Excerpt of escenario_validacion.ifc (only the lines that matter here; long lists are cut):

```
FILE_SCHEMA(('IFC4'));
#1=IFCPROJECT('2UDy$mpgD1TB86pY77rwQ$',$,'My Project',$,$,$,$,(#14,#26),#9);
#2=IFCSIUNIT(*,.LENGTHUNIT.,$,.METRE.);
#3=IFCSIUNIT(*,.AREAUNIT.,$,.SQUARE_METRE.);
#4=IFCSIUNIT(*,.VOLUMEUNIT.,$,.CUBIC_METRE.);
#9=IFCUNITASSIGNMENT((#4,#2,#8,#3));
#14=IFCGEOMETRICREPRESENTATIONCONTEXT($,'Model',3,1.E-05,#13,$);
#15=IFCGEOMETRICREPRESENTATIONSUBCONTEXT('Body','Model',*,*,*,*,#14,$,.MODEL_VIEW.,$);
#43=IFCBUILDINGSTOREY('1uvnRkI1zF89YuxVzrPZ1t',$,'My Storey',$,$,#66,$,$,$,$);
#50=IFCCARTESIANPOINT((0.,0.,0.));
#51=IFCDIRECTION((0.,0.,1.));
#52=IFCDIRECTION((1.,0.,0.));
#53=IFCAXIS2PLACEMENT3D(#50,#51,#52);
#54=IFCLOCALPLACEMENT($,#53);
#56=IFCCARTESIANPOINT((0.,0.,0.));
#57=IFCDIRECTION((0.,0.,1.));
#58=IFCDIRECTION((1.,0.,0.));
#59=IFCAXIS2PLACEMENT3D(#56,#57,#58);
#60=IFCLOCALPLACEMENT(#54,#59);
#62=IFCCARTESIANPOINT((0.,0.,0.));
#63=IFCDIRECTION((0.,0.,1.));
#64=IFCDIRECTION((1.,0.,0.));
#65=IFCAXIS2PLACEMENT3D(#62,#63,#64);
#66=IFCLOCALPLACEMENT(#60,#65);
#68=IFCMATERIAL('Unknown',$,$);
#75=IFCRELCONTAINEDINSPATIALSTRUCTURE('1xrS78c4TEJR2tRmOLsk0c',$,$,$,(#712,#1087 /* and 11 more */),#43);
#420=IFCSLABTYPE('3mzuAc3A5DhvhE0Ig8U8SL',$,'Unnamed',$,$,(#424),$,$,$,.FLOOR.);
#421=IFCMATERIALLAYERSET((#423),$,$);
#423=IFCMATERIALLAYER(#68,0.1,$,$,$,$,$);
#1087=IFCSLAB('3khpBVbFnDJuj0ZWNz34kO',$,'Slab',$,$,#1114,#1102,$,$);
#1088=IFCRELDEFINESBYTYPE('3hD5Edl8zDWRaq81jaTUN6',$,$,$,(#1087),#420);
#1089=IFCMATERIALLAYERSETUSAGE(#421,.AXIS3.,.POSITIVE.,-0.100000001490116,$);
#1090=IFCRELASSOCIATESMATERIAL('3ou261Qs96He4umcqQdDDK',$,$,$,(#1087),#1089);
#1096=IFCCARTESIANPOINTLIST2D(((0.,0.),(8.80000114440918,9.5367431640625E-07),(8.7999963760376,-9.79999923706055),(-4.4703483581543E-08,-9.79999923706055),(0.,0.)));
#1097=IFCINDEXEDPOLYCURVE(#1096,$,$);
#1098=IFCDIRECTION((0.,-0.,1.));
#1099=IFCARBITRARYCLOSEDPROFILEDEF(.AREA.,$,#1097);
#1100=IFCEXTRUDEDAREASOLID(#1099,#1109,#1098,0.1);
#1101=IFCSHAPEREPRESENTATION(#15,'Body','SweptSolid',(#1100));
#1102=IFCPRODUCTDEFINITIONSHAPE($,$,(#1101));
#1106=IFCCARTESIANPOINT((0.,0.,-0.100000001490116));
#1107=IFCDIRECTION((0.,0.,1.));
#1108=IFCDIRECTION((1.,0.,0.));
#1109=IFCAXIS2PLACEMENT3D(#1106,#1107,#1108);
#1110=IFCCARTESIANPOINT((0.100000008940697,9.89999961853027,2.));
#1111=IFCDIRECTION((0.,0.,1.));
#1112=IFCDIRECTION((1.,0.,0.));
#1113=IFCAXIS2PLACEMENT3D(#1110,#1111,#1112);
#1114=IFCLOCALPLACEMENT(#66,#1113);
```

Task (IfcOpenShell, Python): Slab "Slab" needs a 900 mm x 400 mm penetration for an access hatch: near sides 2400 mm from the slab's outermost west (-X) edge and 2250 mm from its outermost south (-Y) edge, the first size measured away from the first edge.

```python
import numpy as np
import ifcopenshell
import ifcopenshell.api.feature
import ifcopenshell.api.geometry
import ifcopenshell.api.root
import ifcopenshell.geom
import ifcopenshell.util.placement
import ifcopenshell.util.representation
import ifcopenshell.util.shape
import ifcopenshell.util.unit

model = ifcopenshell.open("escenario_validacion.ifc")
unit_scale = ifcopenshell.util.unit.calculate_unit_scale(model)
settings = ifcopenshell.geom.settings()


def volume(element):
    """Net volume in cubic metres, openings subtracted."""
    shape = ifcopenshell.geom.create_shape(settings, element)
    return ifcopenshell.util.shape.get_volume(shape.geometry)


slab = model.by_id(1087)
before = volume(slab)

# Extent in the slab's own axes, in metres. The edges named are its -X and -Y sides.
slab_shape = ifcopenshell.geom.create_shape(settings, slab)
vertices = ifcopenshell.util.shape.get_vertices(slab_shape.geometry)
x_min, y_min, bottom = vertices.min(axis=0)
top = vertices[:, 2].max()

opening = ifcopenshell.api.root.create_entity(model, ifc_class="IfcOpeningElement", name="Access hatch opening", predefined_type="OPENING")
context = ifcopenshell.util.representation.get_context(model, "Model", "Body", "MODEL_VIEW")
width, depth = 0.9, 0.4
outline = [(0.0, 0.0), (width, 0.0), (width, depth), (0.0, depth), (0.0, 0.0)]
# Overshoot both faces by 50 mm so the cut is clean.
shape = ifcopenshell.api.geometry.add_slab_representation(
    model, context=context, depth=top - bottom + 0.1, polyline=outline
)
ifcopenshell.api.geometry.assign_representation(model, product=opening, representation=shape)

matrix = ifcopenshell.util.placement.get_local_placement(slab.ObjectPlacement)
matrix[:, 3] = matrix @ np.append(np.array([x_min + 2.4, y_min + 2.25, bottom - 0.05]) / unit_scale, 1.0)
ifcopenshell.api.geometry.edit_object_placement(model, product=opening, matrix=matrix, is_si=False)
ifcopenshell.api.feature.add_feature(model, feature=opening, element=slab)

after = volume(slab)

print(f"slab volume {before:.3f} -> {after:.3f} m3")

model.write("escenario_validacion_edited.ifc")
```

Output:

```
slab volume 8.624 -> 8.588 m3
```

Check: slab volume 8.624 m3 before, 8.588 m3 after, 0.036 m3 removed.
